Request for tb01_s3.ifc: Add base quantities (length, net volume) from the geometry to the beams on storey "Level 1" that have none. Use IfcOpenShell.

First a look at what the model holds.

```python
import ifcopenshell
import ifcopenshell.util.element
import ifcopenshell.util.unit

model = ifcopenshell.open("tb01_s3.ifc")
print(model.schema)
for unit_type in ("LENGTHUNIT", "AREAUNIT", "VOLUMEUNIT"):
    print(unit_type, ifcopenshell.util.unit.calculate_unit_scale(model, unit_type))
storey = next(s for s in model.by_type("IfcBuildingStorey") if s.Name == "Level 1")
beams = [e for e in ifcopenshell.util.element.get_decomposition(storey) if e.is_a("IfcBeam")]
for e in sorted(beams, key=lambda e: e.id()):
    print(e.id(), e.is_a(), e.Name, list(ifcopenshell.util.element.get_psets(e, qtos_only=True)), sep=" | ")
```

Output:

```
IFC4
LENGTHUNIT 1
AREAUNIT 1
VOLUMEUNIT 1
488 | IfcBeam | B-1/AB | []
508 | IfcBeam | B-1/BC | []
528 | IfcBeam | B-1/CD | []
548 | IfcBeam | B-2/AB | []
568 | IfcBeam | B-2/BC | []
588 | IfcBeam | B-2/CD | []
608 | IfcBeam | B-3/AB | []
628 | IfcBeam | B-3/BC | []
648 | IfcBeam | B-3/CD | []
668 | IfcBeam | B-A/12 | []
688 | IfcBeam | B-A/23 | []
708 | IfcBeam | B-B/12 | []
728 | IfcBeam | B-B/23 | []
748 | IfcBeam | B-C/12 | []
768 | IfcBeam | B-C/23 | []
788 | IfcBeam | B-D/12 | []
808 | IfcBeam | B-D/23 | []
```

```python
import ifcopenshell
import ifcopenshell.api.pset
import ifcopenshell.geom
import ifcopenshell.util.element
import ifcopenshell.util.shape
import ifcopenshell.util.unit

model = ifcopenshell.open("tb01_s3.ifc")
unit_scale = ifcopenshell.util.unit.calculate_unit_scale(model)
volume_scale = ifcopenshell.util.unit.calculate_unit_scale(model, "VOLUMEUNIT")
settings = ifcopenshell.geom.settings()

storey = next(s for s in model.by_type("IfcBuildingStorey") if s.Name == "Level 1")
beams = [e for e in ifcopenshell.util.element.get_decomposition(storey) if e.is_a("IfcBeam")]

for e in sorted(beams, key=lambda e: e.id()):
    if ifcopenshell.util.element.get_psets(e, qtos_only=True, should_inherit=False):
        continue
    # Geometry comes back in metres, in the element's own axes.
    shape = ifcopenshell.geom.create_shape(settings, e)
    values = {
        "Length": ifcopenshell.util.shape.get_max_xyz(shape.geometry) / unit_scale,
        "NetVolume": ifcopenshell.util.shape.get_volume(shape.geometry) / volume_scale,
    }
    qto = ifcopenshell.api.pset.add_qto(model, product=e, name="Qto_BeamBaseQuantities")
    ifcopenshell.api.pset.edit_qto(model, qto=qto, properties=values)
    print(e.id(), {k: round(v, 3) for k, v in values.items()})

model.write("tb01_s3_updated.ifc")
```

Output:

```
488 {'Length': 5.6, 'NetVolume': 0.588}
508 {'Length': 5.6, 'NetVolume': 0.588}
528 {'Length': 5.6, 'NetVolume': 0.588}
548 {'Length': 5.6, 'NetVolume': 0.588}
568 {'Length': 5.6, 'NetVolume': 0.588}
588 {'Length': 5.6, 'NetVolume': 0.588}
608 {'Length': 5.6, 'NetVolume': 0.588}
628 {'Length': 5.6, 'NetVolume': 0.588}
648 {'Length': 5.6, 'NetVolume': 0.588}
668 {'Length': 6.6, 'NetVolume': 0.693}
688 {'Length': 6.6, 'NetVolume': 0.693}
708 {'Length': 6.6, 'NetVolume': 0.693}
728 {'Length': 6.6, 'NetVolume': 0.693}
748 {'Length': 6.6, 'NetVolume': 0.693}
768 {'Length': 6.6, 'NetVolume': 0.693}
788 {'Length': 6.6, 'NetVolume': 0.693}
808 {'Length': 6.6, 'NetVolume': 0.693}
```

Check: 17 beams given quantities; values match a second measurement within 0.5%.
